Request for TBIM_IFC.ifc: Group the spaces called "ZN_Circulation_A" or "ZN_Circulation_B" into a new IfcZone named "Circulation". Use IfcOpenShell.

First a look at what the model holds.

```python
import ifcopenshell

model = ifcopenshell.open("TBIM_IFC.ifc")
print(model.schema)
seen = {}
for space in model.by_type("IfcSpace"):
    seen[space.LongName] = seen.get(space.LongName, 0) + 1
for name, count in sorted(seen.items(), key=str):
    print(count, "x", name)
print("zones:", [z.Name for z in model.by_type("IfcZone")][:20])
```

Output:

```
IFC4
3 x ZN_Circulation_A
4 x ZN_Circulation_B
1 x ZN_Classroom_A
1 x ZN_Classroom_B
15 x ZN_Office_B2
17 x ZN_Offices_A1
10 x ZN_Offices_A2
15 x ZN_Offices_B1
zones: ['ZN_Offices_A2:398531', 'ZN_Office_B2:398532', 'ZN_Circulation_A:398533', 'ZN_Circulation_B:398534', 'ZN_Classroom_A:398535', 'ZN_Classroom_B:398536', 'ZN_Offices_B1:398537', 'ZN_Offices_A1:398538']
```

```python
import ifcopenshell
import ifcopenshell.api.group
import ifcopenshell.api.root

model = ifcopenshell.open("TBIM_IFC.ifc")

names = {"ZN_Circulation_A", "ZN_Circulation_B"}
spaces = [s for s in model.by_type("IfcSpace") if s.LongName in names]

zone = ifcopenshell.api.root.create_entity(model, ifc_class="IfcZone", name="Circulation")
ifcopenshell.api.group.assign_group(model, products=spaces, group=zone)
print(len(spaces), "spaces in", zone.Name)

model.write("TBIM_IFC_v2.ifc")
```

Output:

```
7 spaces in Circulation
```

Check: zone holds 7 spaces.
